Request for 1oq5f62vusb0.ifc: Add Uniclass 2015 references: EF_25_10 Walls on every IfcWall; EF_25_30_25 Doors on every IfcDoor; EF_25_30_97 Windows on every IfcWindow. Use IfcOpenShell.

First a look at what the model holds.

```python
import ifcopenshell

model = ifcopenshell.open("1oq5f62vusb0.ifc")
print(model.schema)
print("classifications:", [c.Name for c in model.by_type("IfcClassification")])
for ifc_class in ("IfcDoor", "IfcRoof", "IfcStair", "IfcWall", "IfcWindow"):
    print(ifc_class, len(model.by_type(ifc_class)))
```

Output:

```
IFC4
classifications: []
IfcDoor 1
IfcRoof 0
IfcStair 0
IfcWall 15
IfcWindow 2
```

```python
import ifcopenshell
import ifcopenshell.api.classification

model = ifcopenshell.open("1oq5f62vusb0.ifc")

system = ifcopenshell.api.classification.add_classification(model, classification="Uniclass 2015")

codes = {
    "IfcWall": ("EF_25_10", "Walls"),
    "IfcDoor": ("EF_25_30_25", "Doors"),
    "IfcWindow": ("EF_25_30_97", "Windows"),
}
for ifc_class, (code, name) in codes.items():
    products = model.by_type(ifc_class)
    ifcopenshell.api.classification.add_reference(
        model, products=products, classification=system, identification=code, name=name
    )
    print(code, len(products))

model.write("1oq5f62vusb0_rev.ifc")
```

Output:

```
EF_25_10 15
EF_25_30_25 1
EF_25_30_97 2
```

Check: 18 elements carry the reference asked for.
